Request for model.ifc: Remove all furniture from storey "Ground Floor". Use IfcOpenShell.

First a look at what the model holds.

```python
import ifcopenshell
import ifcopenshell.util.element

model = ifcopenshell.open("model.ifc")
print(model.schema)
storey = next(s for s in model.by_type("IfcBuildingStorey") if s.Name == "Ground Floor")
furniture = [e for e in ifcopenshell.util.element.get_decomposition(storey) if e.is_a("IfcFurnishingElement")]
seen = {}
for e in furniture:
    element_type = ifcopenshell.util.element.get_type(e)
    name = element_type.Name if element_type not in (None, e) else None
    seen[name] = seen.get(name, 0) + 1
for name, count in sorted(seen.items(), key=str):
    print(count, "x", name)
```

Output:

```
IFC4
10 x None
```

```python
import ifcopenshell
import ifcopenshell.api.root
import ifcopenshell.util.element

model = ifcopenshell.open("model.ifc")

storey = next(s for s in model.by_type("IfcBuildingStorey") if s.Name == "Ground Floor")
furniture = [e for e in ifcopenshell.util.element.get_decomposition(storey) if e.is_a("IfcFurnishingElement")]

for e in furniture:
    ifcopenshell.api.root.remove_product(model, product=e)
print(len(furniture), "removed")

model.write("model_v2.ifc")
```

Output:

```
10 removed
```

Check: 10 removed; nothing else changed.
